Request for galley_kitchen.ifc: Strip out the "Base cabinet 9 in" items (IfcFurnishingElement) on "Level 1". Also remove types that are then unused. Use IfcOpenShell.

First a look at what the model holds.

```python
import ifcopenshell
import ifcopenshell.util.element

model = ifcopenshell.open("galley_kitchen.ifc")
print(model.schema)
storey = next(s for s in model.by_type("IfcBuildingStorey") if s.Name == "Level 1")
furniture = [e for e in ifcopenshell.util.element.get_decomposition(storey) if e.is_a("IfcFurnishingElement")]
seen = {}
for e in furniture:
    element_type = ifcopenshell.util.element.get_type(e)
    name = element_type.Name if element_type not in (None, e) else None
    seen[name] = seen.get(name, 0) + 1
for name, count in sorted(seen.items(), key=str):
    print(count, "x", name)
```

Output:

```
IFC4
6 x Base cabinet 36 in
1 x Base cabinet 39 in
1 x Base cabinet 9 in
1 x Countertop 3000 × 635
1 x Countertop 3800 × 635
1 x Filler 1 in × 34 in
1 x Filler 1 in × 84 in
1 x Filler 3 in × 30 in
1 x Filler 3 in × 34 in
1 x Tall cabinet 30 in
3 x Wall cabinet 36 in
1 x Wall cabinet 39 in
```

```python
import ifcopenshell
import ifcopenshell.api.root
import ifcopenshell.util.element

model = ifcopenshell.open("galley_kitchen.ifc")

storey = next(s for s in model.by_type("IfcBuildingStorey") if s.Name == "Level 1")
furniture = [e for e in ifcopenshell.util.element.get_decomposition(storey) if e.is_a("IfcFurnishingElement")]
targets = [e for e in furniture if (t := ifcopenshell.util.element.get_type(e)) not in (None, e) and t.Name == "Base cabinet 9 in"]
types = {ifcopenshell.util.element.get_type(e) for e in targets} - {None, *targets}

for e in targets:
    ifcopenshell.api.root.remove_product(model, product=e)
print(len(targets), "removed")

unused = [t for t in types if not ifcopenshell.util.element.get_types(t)]
for t in unused:
    ifcopenshell.api.root.remove_product(model, product=t)
print(len(unused), "unused types removed")

model.write("galley_kitchen_edited.ifc")
```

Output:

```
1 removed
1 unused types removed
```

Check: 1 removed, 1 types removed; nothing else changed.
